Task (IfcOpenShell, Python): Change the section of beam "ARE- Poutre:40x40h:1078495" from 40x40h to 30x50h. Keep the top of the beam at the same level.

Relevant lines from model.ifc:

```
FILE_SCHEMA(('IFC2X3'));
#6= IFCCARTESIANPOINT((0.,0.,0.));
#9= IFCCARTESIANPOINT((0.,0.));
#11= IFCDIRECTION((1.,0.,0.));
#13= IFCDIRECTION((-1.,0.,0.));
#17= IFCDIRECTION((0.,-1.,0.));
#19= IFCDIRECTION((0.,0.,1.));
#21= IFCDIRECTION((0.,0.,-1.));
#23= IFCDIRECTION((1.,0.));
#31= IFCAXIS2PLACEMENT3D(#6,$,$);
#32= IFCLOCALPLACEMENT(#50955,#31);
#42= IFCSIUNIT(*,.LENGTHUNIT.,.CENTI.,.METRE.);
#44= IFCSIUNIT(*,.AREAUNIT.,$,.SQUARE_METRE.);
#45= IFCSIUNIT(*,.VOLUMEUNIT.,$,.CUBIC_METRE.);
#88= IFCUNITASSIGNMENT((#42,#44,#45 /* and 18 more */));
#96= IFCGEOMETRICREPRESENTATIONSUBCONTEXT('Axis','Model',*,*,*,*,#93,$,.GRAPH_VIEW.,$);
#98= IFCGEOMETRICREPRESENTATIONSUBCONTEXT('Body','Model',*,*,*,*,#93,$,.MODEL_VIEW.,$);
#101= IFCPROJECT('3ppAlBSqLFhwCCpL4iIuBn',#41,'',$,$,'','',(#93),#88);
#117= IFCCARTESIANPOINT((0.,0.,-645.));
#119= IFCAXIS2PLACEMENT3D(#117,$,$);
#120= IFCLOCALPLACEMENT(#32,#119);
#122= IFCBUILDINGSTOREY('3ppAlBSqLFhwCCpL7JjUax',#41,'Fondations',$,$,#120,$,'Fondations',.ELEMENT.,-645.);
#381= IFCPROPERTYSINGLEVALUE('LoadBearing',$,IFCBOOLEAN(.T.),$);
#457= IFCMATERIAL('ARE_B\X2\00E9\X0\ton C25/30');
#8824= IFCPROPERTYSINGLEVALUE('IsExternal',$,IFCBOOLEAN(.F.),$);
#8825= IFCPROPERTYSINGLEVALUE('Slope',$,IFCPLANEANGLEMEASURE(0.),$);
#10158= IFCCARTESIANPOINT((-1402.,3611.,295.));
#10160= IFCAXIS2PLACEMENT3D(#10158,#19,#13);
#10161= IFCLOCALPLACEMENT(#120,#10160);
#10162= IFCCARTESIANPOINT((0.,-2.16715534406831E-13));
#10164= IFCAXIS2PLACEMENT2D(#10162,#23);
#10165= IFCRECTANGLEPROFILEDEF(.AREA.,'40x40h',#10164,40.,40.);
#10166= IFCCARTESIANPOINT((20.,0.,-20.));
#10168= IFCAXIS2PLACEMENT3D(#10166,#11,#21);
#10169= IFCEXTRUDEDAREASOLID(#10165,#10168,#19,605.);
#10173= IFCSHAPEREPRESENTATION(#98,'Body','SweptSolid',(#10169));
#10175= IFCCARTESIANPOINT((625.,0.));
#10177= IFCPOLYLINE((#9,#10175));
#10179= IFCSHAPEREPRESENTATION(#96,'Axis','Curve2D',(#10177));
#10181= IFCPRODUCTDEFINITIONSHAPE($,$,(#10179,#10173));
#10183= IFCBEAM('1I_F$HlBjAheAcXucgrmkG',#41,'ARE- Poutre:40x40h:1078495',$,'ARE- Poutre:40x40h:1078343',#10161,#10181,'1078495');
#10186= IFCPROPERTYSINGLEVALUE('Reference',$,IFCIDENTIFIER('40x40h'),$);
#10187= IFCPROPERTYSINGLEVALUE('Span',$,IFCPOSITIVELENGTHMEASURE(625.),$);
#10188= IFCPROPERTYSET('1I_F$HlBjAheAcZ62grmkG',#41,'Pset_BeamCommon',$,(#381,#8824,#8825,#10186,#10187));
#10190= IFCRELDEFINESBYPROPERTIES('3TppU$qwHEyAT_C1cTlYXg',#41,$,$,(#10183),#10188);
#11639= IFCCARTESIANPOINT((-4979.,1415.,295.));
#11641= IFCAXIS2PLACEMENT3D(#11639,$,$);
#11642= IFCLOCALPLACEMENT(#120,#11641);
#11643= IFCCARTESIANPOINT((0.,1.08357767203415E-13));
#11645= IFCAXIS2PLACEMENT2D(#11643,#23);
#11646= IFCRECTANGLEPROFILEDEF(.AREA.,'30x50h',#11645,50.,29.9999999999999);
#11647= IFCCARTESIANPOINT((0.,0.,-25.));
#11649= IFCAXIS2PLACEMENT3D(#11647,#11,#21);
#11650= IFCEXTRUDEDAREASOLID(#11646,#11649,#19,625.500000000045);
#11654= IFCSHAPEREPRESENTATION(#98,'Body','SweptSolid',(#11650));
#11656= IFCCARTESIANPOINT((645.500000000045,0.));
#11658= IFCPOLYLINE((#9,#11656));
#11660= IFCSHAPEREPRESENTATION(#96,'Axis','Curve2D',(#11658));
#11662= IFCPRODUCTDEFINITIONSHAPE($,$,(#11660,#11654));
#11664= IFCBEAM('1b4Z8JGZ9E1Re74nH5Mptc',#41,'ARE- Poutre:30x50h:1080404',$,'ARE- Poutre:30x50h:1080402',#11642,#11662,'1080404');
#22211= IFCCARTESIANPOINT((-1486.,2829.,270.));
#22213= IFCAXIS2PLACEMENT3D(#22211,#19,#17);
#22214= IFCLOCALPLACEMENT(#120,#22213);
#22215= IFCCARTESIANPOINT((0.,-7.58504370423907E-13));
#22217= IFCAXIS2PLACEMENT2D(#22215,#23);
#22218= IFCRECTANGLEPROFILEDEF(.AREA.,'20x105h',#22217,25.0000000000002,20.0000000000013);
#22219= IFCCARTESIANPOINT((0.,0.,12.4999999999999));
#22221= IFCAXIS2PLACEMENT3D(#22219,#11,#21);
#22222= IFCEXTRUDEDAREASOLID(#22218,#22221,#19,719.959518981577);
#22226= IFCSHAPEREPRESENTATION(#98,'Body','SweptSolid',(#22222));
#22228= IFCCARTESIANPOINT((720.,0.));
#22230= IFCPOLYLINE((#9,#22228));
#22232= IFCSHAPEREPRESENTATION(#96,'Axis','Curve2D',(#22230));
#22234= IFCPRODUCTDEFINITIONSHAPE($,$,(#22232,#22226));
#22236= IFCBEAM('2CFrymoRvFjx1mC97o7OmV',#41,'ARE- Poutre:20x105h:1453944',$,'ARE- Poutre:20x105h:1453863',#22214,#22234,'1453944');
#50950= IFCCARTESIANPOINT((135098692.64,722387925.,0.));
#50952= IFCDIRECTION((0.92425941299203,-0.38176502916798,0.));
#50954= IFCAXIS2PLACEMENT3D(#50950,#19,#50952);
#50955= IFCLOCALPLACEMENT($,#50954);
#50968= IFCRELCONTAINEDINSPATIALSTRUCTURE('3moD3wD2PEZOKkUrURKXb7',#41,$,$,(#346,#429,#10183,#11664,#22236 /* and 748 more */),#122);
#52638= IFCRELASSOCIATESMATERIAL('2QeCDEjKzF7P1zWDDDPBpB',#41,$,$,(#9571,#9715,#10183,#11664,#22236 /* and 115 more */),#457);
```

```python
import ifcopenshell
import ifcopenshell.api.pset
import ifcopenshell.util.element
import ifcopenshell.util.representation

model = ifcopenshell.open("model.ifc")

member = model.by_guid("1I_F$HlBjAheAcXucgrmkG")
source = next(p for p in model.by_type("IfcRectangleProfileDef") if p.ProfileName == "30x50h")

body = ifcopenshell.util.representation.get_representation(member, "Model", "Body")
solid = body.Items[0]
old_profile = solid.SweptArea

# Copy the section's sizes but keep this member's own profile position.
profile = ifcopenshell.util.element.copy(model, source)
# Profiles are centred, so shift by half the change in depth to hold the top.
shift = (old_profile.XDim - profile.XDim) / 2
x, y = old_profile.Position.Location.Coordinates
up = (-1.0, 0.0)  # upwards, in the solid's own plane
location = model.createIfcCartesianPoint((x + up[0] * shift, y + up[1] * shift))
profile.Position = model.createIfcAxis2Placement2D(location, old_profile.Position.RefDirection)
solid.SweptArea = profile
if not model.get_total_inverses(old_profile):
    ifcopenshell.util.element.remove_deep2(model, old_profile)
member.Name = member.Name.replace("40x40h", "30x50h")
member.ObjectType = member.ObjectType.replace("40x40h", "30x50h")
pset = model.by_id(ifcopenshell.util.element.get_pset(member, "Pset_BeamCommon", should_inherit=False)["id"])
ifcopenshell.api.pset.edit_pset(model, pset=pset, properties={"Reference": "30x50h"})

print(solid.SweptArea)

model.write("model_v2.ifc")
```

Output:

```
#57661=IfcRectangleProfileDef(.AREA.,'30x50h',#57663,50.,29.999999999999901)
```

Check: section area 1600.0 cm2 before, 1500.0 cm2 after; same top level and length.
